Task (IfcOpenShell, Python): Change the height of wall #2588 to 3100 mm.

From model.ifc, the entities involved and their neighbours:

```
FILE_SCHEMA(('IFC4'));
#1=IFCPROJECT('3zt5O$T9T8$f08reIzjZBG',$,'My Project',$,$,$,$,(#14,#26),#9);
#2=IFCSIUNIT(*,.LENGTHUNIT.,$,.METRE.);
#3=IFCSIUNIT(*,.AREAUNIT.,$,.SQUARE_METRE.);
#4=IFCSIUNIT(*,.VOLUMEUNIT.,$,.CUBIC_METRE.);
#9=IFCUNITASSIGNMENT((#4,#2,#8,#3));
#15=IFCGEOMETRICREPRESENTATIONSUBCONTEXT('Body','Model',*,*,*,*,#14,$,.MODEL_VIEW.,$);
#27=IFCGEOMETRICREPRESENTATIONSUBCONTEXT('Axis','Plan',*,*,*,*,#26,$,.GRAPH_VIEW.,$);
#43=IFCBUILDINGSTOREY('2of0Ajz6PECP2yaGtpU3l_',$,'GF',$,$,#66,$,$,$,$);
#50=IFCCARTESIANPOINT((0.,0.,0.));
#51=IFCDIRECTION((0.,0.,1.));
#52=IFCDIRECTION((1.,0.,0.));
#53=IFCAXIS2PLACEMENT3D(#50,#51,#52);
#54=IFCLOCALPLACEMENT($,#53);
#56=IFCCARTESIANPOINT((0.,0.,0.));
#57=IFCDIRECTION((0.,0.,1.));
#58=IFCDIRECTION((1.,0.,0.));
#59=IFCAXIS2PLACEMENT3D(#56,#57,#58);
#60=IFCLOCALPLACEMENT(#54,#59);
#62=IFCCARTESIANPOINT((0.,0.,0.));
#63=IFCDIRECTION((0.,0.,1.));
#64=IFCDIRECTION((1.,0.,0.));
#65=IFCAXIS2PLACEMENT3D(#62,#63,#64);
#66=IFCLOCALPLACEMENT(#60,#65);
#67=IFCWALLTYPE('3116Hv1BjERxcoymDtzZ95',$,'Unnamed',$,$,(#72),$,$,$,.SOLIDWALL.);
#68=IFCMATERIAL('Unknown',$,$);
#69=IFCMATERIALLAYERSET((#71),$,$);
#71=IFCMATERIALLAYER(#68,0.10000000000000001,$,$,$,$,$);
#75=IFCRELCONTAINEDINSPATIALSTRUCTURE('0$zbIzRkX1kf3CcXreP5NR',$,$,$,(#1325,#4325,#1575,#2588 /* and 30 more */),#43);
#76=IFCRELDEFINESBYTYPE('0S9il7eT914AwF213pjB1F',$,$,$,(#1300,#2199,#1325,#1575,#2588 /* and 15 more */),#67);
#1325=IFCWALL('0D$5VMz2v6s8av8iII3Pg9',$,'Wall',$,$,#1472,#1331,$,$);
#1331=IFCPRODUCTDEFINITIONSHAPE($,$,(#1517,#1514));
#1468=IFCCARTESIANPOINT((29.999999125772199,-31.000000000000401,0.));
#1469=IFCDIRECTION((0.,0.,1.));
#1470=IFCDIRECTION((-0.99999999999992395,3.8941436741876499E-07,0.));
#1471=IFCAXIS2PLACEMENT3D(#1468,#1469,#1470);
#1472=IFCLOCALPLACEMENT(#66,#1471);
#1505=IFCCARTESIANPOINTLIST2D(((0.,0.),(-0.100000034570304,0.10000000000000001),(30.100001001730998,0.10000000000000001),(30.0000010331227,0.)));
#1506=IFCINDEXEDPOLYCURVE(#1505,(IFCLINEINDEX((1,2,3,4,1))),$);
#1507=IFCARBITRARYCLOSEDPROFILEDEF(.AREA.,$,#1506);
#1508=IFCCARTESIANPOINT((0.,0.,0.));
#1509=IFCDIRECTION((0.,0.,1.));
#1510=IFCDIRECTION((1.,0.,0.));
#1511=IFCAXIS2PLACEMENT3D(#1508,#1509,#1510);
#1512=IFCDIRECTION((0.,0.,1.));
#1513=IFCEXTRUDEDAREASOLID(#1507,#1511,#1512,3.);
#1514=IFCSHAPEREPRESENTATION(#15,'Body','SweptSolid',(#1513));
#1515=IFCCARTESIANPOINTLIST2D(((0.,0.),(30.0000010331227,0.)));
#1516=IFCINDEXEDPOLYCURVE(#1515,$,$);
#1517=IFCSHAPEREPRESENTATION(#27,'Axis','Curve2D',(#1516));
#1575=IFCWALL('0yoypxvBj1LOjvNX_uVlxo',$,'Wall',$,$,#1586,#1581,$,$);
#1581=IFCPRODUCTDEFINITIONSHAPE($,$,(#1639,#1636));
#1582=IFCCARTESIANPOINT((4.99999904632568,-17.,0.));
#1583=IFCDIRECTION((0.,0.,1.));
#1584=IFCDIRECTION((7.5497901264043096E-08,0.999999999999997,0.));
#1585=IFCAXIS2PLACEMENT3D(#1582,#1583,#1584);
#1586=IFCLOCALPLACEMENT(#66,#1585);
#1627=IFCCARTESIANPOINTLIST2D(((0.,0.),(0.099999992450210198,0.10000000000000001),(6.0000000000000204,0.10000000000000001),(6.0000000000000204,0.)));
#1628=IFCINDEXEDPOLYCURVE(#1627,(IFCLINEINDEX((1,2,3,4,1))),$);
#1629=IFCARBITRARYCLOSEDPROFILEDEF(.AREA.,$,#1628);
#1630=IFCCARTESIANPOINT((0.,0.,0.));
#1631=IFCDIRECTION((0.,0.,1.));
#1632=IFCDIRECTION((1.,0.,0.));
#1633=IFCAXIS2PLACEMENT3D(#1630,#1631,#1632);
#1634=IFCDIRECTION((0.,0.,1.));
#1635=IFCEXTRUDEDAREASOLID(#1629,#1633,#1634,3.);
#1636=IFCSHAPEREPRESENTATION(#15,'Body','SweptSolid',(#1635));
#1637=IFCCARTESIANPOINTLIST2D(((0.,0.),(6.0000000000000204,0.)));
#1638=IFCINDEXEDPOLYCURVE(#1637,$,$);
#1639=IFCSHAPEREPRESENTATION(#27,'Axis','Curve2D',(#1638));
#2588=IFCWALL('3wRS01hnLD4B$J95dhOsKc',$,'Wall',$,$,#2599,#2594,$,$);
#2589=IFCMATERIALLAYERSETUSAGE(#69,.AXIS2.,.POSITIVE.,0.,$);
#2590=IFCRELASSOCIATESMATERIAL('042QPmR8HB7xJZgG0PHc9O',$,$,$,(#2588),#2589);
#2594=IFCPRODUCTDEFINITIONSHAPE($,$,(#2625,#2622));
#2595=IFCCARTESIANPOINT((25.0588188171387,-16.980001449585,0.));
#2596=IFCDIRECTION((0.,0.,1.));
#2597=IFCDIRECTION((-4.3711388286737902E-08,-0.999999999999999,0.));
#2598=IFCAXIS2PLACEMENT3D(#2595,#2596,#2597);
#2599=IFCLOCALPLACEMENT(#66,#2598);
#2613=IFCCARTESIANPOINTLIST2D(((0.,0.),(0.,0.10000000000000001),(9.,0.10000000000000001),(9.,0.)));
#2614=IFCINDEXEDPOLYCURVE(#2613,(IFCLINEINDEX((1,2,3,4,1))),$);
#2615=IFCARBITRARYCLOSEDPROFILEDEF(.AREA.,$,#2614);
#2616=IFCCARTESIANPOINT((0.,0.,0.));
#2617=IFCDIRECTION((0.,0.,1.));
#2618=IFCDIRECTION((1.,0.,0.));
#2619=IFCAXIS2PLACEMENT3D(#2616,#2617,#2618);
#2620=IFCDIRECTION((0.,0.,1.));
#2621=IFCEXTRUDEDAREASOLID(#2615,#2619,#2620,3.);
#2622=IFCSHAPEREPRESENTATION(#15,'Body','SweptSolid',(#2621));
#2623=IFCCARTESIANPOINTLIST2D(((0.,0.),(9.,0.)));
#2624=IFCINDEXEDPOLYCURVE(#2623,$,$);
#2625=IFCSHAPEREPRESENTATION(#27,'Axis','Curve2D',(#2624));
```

```python
import ifcopenshell
import ifcopenshell.geom
import ifcopenshell.util.representation
import ifcopenshell.util.shape

model = ifcopenshell.open("model.ifc")
settings = ifcopenshell.geom.settings()


def volume(element):
    """Net volume in cubic metres, openings subtracted."""
    shape = ifcopenshell.geom.create_shape(settings, element)
    return ifcopenshell.util.shape.get_volume(shape.geometry)


wall = model.by_guid("3wRS01hnLD4B$J95dhOsKc")
before = volume(wall)

body = ifcopenshell.util.representation.get_representation(wall, "Model", "Body")
solid = body.Items[0]
old_height = solid.Depth
solid.Depth = 3.1
after = volume(wall)

print(f"height {old_height:g} -> {solid.Depth:g}, volume {before:.3f} -> {after:.3f} m3")

model.write("model_edited.ifc")
```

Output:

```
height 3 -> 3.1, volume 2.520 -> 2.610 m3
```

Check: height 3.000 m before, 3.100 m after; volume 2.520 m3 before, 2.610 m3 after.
